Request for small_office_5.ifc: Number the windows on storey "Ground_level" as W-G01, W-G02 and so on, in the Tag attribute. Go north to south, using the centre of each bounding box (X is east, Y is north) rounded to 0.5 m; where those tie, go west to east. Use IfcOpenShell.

First a look at what the model holds.

```python
import ifcopenshell
import ifcopenshell.util.element
import ifcopenshell.util.placement

model = ifcopenshell.open("small_office_5.ifc")
print(model.schema)
storey = next(s for s in model.by_type("IfcBuildingStorey") if s.Name == "Ground_level")
windows = [e for e in ifcopenshell.util.element.get_decomposition(storey) if e.is_a("IfcWindow")]
for e in sorted(windows, key=lambda e: e.id()):
    origin = ifcopenshell.util.placement.get_local_placement(e.ObjectPlacement)[:3, 3]
    print(e.id(), e.Tag, e.Name, origin.round(2) + 0.0, sep=" | ")
```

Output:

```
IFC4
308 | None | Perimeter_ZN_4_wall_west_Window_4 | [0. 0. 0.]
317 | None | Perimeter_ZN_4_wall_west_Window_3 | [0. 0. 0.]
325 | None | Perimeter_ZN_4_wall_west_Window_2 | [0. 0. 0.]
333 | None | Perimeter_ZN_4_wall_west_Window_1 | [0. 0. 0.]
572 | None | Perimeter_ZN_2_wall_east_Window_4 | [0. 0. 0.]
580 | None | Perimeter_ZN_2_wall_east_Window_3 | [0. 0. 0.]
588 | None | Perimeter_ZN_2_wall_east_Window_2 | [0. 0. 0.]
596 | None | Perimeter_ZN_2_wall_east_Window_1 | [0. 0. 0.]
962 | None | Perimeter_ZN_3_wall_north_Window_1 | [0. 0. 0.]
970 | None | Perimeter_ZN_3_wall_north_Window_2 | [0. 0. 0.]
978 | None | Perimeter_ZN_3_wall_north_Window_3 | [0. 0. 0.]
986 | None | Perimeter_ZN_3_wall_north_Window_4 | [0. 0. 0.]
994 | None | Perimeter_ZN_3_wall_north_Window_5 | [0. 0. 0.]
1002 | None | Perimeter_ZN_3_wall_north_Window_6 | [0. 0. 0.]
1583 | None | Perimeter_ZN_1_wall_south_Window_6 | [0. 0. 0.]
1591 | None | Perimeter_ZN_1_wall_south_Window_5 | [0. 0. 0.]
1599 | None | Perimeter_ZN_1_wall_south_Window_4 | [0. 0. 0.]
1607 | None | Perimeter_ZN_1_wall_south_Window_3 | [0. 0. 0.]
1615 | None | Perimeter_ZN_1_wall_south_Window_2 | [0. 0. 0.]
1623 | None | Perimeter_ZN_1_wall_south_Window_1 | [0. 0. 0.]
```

```python
import ifcopenshell
import ifcopenshell.geom
import ifcopenshell.util.element
import ifcopenshell.util.shape

model = ifcopenshell.open("small_office_5.ifc")
settings = ifcopenshell.geom.settings()
settings.set("use-world-coords", True)


def centre(element):
    shape = ifcopenshell.geom.create_shape(settings, element)
    return ifcopenshell.util.shape.get_bbox_centroid(shape.geometry)


storey = next(s for s in model.by_type("IfcBuildingStorey") if s.Name == "Ground_level")
windows = [e for e in ifcopenshell.util.element.get_decomposition(storey) if e.is_a("IfcWindow")]

# Insertion points can sit at a corner or the storey origin, so sort by the geometry (in metres).
centres = {e: centre(e) for e in windows}
windows.sort(key=lambda e: (-round(centres[e][1] / 0.5), centres[e][0]))

for i, e in enumerate(windows, start=1):
    number = f"W-G{i:02d}"
    e.Tag = number
    print(e.id(), number)

model.write("small_office_5-out.ifc")
```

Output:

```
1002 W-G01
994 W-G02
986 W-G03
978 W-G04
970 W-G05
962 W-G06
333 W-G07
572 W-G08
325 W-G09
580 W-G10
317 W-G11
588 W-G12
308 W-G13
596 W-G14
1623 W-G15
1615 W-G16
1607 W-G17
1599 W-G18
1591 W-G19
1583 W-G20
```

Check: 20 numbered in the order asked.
